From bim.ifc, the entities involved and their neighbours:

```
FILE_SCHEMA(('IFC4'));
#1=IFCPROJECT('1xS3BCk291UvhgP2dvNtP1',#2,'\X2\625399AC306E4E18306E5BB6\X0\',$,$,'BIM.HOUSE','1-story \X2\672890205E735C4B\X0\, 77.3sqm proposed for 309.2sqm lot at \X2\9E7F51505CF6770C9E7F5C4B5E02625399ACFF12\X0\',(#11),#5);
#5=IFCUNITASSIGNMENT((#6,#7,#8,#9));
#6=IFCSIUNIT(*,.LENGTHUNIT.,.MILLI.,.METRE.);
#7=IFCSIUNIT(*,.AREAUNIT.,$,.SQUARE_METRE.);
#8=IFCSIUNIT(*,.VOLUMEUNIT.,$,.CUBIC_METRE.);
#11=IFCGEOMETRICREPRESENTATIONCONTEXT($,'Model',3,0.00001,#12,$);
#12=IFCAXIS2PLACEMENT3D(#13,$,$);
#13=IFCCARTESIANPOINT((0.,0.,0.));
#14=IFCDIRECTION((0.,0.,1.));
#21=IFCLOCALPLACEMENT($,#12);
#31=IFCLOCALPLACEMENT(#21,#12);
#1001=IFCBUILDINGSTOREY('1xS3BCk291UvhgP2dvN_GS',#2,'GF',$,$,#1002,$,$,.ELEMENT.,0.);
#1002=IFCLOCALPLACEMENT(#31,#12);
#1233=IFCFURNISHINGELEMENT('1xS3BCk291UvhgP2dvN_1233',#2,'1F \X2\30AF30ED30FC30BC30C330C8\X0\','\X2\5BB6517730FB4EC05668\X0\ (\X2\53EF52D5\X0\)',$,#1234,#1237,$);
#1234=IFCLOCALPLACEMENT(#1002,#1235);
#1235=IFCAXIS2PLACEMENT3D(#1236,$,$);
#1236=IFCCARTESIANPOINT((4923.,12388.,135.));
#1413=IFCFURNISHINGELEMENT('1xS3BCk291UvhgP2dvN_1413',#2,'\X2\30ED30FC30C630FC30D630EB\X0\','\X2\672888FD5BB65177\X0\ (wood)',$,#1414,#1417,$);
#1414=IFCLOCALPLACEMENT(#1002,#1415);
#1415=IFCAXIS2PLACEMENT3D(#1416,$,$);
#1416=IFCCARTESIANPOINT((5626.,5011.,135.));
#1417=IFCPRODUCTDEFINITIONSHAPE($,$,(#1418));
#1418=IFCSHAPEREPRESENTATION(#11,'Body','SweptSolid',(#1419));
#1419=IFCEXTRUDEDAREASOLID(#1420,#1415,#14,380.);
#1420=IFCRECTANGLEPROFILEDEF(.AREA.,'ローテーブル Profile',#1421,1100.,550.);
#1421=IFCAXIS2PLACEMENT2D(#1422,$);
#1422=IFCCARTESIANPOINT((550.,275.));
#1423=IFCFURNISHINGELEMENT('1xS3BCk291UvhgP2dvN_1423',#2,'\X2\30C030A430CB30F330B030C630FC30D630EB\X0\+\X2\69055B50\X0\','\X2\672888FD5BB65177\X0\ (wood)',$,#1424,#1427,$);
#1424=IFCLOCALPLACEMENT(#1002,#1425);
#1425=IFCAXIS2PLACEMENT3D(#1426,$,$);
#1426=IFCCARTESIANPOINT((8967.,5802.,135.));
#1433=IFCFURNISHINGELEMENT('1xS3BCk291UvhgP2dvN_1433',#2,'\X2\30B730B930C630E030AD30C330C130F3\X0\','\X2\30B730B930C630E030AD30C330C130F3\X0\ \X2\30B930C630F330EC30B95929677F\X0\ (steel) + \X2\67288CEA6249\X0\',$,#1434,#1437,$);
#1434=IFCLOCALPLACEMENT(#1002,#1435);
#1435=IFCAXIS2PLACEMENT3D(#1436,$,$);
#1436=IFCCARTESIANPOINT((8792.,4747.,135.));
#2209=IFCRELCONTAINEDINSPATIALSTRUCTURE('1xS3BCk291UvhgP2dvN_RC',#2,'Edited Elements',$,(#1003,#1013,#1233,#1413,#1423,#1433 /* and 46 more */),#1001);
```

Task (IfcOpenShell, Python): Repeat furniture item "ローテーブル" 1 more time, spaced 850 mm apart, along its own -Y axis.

```python
import ifcopenshell
import ifcopenshell.api.geometry
import ifcopenshell.api.root
import ifcopenshell.util.element
import ifcopenshell.util.placement
import ifcopenshell.util.unit

model = ifcopenshell.open("bim.ifc")
unit_scale = ifcopenshell.util.unit.calculate_unit_scale(model)


def reuse_history(source, copy):
    """copy_class also copies each property set's owner history, people and application; keep the originals."""
    for rel in copy.IsDefinedBy:
        if rel.is_a("IfcRelDefinesByProperties") and (history := rel.RelatingPropertyDefinition.OwnerHistory):
            rel.RelatingPropertyDefinition.OwnerHistory = source.OwnerHistory
            ifcopenshell.util.element.remove_deep2(model, history)


source = model.by_guid("1xS3BCk291UvhgP2dvN_1413")
base = ifcopenshell.util.placement.get_local_placement(source.ObjectPlacement)
step = -base[:3, 1] * 0.85 / unit_scale

for i in range(1, 2):
    copy = ifcopenshell.api.root.copy_class(model, product=source)
    copy.Representation = ifcopenshell.util.element.copy_deep(
        model, source.Representation, exclude=["IfcGeometricRepresentationContext", "IfcRepresentationMap"]
    )
    reuse_history(source, copy)
    matrix = base.copy()
    matrix[:3, 3] += i * step
    print("added at", matrix[:3, 3].round(3) + 0.0)
    ifcopenshell.api.geometry.edit_object_placement(model, product=copy, matrix=matrix, is_si=False)

model.write("bim_v2.ifc")
```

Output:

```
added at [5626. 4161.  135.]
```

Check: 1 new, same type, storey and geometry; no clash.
